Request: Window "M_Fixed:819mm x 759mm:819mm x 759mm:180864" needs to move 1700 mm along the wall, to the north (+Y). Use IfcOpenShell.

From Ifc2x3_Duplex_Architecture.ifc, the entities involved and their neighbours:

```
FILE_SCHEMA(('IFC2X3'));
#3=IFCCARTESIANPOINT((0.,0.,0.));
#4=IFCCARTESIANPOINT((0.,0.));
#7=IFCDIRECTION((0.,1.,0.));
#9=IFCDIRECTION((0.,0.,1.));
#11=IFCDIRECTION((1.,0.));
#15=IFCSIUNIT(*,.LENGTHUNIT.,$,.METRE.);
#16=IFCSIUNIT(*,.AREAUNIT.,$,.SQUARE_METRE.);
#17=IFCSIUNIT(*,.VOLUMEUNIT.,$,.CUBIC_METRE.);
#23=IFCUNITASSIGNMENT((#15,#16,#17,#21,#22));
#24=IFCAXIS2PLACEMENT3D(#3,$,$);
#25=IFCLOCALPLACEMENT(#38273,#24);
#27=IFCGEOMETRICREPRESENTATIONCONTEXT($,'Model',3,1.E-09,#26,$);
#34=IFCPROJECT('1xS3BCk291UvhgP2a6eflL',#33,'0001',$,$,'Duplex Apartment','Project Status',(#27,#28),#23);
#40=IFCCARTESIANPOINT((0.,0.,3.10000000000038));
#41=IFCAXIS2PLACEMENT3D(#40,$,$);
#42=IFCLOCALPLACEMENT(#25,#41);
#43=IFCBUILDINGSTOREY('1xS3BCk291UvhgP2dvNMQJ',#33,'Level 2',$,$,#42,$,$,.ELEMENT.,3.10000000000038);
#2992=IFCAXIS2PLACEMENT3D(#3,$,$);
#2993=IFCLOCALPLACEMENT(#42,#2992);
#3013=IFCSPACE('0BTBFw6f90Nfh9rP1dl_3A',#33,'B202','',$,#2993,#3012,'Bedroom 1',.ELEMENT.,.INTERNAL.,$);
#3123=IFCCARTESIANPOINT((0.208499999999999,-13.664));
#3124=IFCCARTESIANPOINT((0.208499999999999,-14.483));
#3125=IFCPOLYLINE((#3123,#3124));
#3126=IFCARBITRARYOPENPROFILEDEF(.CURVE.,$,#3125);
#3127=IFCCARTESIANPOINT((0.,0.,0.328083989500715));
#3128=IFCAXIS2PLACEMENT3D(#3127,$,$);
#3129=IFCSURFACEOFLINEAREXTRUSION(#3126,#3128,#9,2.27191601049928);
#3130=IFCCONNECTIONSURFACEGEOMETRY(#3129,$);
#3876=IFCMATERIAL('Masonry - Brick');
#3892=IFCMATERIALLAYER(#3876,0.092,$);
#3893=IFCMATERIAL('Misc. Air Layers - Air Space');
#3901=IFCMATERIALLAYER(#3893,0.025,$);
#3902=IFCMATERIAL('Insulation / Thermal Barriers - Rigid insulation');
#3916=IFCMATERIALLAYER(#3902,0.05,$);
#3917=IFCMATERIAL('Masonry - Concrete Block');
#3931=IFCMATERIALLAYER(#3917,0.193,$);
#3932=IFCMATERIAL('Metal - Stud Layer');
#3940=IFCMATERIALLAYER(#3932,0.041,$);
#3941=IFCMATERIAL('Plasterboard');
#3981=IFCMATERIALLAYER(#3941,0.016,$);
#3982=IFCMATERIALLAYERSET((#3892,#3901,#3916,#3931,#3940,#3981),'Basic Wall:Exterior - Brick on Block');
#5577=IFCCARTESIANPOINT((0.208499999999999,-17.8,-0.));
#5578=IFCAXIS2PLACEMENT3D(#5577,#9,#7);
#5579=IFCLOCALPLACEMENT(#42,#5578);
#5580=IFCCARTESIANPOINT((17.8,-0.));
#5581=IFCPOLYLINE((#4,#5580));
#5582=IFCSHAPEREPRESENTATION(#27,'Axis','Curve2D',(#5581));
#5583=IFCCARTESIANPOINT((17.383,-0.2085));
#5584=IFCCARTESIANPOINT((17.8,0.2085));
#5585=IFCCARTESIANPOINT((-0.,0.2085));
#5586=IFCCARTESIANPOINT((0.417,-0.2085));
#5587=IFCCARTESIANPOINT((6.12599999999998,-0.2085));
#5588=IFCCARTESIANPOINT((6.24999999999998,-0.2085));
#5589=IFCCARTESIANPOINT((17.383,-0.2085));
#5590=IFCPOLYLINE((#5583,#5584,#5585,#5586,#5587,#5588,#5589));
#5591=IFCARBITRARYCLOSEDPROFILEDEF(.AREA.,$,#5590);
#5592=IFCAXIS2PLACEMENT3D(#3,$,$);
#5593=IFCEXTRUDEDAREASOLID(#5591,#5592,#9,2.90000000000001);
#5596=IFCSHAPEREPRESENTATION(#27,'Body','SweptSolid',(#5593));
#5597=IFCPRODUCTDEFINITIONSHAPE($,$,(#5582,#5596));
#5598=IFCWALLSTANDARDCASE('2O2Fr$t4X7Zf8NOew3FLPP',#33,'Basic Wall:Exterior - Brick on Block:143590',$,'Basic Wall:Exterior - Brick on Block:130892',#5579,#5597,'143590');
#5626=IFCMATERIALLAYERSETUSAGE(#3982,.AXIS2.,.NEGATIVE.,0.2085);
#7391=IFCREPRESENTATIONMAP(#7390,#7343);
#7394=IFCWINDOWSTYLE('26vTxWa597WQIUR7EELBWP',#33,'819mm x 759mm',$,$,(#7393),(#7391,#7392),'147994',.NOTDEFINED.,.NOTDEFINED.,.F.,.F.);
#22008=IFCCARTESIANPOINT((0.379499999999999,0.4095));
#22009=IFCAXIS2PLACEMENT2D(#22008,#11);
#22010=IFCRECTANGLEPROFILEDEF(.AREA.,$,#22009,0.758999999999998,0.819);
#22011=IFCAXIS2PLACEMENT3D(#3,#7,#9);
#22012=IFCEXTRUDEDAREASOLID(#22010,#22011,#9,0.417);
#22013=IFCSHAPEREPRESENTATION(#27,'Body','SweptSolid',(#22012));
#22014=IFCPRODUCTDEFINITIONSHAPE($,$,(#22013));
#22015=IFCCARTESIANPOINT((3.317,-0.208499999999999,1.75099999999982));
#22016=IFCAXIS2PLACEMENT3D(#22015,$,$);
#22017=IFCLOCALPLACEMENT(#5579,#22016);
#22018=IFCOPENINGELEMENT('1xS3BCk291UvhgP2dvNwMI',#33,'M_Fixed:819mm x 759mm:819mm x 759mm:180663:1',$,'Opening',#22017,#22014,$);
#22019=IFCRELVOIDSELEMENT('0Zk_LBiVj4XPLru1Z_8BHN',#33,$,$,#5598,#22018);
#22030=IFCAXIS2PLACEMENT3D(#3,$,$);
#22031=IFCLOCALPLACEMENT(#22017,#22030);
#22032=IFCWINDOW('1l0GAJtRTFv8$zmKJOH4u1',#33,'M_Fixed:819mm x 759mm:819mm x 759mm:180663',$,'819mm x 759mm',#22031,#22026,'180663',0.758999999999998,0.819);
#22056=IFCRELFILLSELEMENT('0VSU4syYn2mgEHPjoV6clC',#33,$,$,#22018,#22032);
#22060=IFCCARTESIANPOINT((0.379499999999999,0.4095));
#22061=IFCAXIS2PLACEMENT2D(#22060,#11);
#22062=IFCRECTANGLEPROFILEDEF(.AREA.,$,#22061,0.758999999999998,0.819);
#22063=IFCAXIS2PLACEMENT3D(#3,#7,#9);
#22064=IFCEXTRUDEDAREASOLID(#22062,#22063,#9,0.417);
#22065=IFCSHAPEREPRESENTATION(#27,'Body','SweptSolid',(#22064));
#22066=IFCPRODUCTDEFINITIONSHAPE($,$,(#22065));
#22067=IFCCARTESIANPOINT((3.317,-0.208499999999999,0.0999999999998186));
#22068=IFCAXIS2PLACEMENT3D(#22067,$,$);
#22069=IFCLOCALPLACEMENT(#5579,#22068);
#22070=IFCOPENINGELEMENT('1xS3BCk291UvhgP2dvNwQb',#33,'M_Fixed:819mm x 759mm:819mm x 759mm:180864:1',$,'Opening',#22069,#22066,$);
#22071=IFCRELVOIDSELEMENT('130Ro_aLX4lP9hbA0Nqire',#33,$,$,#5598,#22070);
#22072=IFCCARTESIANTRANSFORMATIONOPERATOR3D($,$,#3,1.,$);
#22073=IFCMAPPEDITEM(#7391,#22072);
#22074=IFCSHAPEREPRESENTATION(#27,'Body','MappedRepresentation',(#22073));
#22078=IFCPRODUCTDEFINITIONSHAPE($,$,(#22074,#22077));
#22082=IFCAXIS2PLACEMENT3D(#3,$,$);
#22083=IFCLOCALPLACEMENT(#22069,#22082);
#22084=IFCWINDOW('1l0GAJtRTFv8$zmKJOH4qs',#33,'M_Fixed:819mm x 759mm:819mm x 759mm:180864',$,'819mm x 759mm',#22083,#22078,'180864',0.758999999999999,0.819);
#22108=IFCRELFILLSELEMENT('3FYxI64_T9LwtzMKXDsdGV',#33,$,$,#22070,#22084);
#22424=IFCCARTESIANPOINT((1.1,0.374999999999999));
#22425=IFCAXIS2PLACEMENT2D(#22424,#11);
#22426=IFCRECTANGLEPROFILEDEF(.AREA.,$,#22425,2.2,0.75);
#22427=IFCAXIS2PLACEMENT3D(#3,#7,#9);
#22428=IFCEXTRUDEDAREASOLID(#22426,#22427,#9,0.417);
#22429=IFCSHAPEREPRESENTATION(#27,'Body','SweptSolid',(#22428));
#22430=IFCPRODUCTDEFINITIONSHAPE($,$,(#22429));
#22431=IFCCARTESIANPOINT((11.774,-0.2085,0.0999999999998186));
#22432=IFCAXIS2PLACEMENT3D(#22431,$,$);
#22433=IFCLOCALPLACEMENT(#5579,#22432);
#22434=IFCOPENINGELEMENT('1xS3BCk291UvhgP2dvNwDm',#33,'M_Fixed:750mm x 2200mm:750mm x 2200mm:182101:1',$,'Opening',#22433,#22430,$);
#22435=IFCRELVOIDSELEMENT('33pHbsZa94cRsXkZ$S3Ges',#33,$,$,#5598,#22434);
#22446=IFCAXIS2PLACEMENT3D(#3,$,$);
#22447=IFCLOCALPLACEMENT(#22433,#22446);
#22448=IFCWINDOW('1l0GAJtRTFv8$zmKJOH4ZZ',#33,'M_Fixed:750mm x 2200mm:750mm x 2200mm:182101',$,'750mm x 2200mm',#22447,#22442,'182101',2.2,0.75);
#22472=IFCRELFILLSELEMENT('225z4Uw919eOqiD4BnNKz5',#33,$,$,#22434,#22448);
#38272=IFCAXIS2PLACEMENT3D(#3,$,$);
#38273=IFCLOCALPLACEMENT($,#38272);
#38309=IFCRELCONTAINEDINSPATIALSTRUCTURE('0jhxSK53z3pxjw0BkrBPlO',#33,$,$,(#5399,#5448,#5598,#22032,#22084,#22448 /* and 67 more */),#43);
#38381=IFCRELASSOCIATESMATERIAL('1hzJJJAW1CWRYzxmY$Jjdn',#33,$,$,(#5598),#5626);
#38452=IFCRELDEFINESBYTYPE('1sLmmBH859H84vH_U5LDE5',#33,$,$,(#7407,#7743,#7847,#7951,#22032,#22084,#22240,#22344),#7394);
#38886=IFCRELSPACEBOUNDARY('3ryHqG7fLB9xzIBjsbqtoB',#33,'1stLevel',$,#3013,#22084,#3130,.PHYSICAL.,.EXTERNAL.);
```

```python
import numpy as np
import ifcopenshell
import ifcopenshell.api.geometry
import ifcopenshell.util.placement
import ifcopenshell.util.unit

model = ifcopenshell.open("Ifc2x3_Duplex_Architecture.ifc")
unit_scale = ifcopenshell.util.unit.calculate_unit_scale(model)

window = model.by_guid("1l0GAJtRTFv8$zmKJOH4qs")
opening = window.FillsVoids[0].RelatingOpeningElement
wall = opening.VoidsElements[0].RelatingBuildingElement

wall_matrix = ifcopenshell.util.placement.get_local_placement(wall.ObjectPlacement)
shift = wall_matrix[:3, 0] * 1.7 / unit_scale
before = ifcopenshell.util.placement.get_local_placement(window.ObjectPlacement)[:3, 3].copy()

# The window is placed relative to its opening, so it follows when the opening moves.
matrix = ifcopenshell.util.placement.get_local_placement(opening.ObjectPlacement)
matrix[:3, 3] += shift
ifcopenshell.api.geometry.edit_object_placement(
    model, product=opening, matrix=matrix, is_si=False, should_transform_children=True
)

# Space boundary surfaces are stored in each space's coordinates; move them too.
for rel in window.ProvidesBoundaries:
    if not rel.ConnectionGeometry:
        continue
    surface = rel.ConnectionGeometry.SurfaceOnRelatingElement
    space_matrix = ifcopenshell.util.placement.get_local_placement(rel.RelatingSpace.ObjectPlacement)
    point = np.array(surface.Position.Location.Coordinates) + space_matrix[:3, :3].T @ shift
    surface.Position = model.createIfcAxis2Placement3D(
        model.createIfcCartesianPoint(point.tolist()), surface.Position.Axis, surface.Position.RefDirection
    )

after = ifcopenshell.util.placement.get_local_placement(window.ObjectPlacement)[:3, 3]
print("window moved by", (after - before).round(3) + 0.0)

model.write("Ifc2x3_Duplex_Architecture_updated.ifc")
```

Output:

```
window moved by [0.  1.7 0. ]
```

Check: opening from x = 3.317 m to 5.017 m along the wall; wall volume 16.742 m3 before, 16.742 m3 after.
